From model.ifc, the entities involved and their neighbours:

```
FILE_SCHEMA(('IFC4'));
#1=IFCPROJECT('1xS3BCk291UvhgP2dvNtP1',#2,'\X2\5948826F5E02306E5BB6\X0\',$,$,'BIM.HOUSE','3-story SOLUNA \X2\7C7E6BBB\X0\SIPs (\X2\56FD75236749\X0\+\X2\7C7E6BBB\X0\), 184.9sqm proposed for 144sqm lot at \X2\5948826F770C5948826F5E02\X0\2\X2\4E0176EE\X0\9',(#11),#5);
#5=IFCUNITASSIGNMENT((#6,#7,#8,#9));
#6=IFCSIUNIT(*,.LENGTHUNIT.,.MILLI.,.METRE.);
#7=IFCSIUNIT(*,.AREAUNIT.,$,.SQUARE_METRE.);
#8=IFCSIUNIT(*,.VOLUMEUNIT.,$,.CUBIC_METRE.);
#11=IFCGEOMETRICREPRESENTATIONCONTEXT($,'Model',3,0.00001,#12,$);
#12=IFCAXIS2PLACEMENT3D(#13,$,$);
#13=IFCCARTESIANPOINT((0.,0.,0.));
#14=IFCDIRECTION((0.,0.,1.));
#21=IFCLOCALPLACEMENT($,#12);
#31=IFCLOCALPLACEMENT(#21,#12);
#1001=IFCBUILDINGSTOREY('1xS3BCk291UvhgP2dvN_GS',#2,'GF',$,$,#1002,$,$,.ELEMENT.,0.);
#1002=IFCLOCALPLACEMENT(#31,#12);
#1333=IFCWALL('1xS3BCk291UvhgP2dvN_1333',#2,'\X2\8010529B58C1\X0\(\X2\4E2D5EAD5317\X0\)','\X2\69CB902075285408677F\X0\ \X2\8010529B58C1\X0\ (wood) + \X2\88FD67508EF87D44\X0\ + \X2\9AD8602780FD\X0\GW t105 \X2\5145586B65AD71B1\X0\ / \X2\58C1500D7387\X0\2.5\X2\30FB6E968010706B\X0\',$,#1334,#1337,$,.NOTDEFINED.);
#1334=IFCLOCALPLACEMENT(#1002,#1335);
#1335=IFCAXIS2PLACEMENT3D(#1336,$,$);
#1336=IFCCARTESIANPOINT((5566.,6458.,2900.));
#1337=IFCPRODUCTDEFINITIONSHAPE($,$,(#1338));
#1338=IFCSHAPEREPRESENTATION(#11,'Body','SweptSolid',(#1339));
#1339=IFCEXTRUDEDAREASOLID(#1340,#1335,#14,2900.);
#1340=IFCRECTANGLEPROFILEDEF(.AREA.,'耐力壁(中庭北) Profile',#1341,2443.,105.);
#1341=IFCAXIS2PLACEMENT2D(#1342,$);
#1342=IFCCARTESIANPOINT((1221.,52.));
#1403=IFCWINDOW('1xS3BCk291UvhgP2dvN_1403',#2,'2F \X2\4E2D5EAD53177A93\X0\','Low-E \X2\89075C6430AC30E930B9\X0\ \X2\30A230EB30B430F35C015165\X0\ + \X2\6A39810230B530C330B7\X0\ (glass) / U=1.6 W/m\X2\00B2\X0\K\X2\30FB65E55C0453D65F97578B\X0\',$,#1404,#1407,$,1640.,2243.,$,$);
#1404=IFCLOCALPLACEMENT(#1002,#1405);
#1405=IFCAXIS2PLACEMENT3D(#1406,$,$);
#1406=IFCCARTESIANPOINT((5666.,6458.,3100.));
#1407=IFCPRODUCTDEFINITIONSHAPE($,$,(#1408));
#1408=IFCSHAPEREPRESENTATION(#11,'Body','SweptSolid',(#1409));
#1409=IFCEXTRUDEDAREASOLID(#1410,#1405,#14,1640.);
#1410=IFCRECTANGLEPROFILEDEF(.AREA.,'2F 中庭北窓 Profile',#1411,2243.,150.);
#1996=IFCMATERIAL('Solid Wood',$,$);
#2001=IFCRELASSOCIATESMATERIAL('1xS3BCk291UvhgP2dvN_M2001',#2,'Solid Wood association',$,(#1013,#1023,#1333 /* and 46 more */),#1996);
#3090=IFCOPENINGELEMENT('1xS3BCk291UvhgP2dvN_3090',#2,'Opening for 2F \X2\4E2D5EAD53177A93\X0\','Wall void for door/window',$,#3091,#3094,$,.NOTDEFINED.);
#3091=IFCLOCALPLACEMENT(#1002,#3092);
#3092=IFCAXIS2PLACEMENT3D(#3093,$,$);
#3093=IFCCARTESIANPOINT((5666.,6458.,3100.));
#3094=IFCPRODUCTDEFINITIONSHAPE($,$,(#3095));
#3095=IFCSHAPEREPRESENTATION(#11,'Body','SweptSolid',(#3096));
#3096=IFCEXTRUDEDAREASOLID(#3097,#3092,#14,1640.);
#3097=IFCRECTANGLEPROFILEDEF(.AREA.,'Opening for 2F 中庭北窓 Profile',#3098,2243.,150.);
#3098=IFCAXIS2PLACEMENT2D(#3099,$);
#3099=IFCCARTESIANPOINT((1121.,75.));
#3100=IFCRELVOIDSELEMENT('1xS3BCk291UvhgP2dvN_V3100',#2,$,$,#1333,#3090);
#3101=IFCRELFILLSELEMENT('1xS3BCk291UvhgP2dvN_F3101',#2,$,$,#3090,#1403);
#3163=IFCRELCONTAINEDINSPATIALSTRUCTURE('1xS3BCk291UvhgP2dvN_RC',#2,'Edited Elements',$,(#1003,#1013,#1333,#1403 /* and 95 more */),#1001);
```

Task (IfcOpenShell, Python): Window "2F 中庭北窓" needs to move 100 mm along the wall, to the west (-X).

```python
import ifcopenshell
import ifcopenshell.api.geometry
import ifcopenshell.util.placement
import ifcopenshell.util.unit

model = ifcopenshell.open("model.ifc")
unit_scale = ifcopenshell.util.unit.calculate_unit_scale(model)

window = model.by_id(1403)
opening = window.FillsVoids[0].RelatingOpeningElement
wall = opening.VoidsElements[0].RelatingBuildingElement

wall_matrix = ifcopenshell.util.placement.get_local_placement(wall.ObjectPlacement)
shift = wall_matrix[:3, 0] * -0.1 / unit_scale
before = ifcopenshell.util.placement.get_local_placement(window.ObjectPlacement)[:3, 3].copy()

# The window is not placed relative to its opening, so move both.
for product in (opening, window):
    matrix = ifcopenshell.util.placement.get_local_placement(product.ObjectPlacement)
    matrix[:3, 3] += shift
    ifcopenshell.api.geometry.edit_object_placement(model, product=product, matrix=matrix, is_si=False)

after = ifcopenshell.util.placement.get_local_placement(window.ObjectPlacement)[:3, 3]
print("window moved by", (after - before).round(3) + 0.0)

model.write("model_edited.ifc")
```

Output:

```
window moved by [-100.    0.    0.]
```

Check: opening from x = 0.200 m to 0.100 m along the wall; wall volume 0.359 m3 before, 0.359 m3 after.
